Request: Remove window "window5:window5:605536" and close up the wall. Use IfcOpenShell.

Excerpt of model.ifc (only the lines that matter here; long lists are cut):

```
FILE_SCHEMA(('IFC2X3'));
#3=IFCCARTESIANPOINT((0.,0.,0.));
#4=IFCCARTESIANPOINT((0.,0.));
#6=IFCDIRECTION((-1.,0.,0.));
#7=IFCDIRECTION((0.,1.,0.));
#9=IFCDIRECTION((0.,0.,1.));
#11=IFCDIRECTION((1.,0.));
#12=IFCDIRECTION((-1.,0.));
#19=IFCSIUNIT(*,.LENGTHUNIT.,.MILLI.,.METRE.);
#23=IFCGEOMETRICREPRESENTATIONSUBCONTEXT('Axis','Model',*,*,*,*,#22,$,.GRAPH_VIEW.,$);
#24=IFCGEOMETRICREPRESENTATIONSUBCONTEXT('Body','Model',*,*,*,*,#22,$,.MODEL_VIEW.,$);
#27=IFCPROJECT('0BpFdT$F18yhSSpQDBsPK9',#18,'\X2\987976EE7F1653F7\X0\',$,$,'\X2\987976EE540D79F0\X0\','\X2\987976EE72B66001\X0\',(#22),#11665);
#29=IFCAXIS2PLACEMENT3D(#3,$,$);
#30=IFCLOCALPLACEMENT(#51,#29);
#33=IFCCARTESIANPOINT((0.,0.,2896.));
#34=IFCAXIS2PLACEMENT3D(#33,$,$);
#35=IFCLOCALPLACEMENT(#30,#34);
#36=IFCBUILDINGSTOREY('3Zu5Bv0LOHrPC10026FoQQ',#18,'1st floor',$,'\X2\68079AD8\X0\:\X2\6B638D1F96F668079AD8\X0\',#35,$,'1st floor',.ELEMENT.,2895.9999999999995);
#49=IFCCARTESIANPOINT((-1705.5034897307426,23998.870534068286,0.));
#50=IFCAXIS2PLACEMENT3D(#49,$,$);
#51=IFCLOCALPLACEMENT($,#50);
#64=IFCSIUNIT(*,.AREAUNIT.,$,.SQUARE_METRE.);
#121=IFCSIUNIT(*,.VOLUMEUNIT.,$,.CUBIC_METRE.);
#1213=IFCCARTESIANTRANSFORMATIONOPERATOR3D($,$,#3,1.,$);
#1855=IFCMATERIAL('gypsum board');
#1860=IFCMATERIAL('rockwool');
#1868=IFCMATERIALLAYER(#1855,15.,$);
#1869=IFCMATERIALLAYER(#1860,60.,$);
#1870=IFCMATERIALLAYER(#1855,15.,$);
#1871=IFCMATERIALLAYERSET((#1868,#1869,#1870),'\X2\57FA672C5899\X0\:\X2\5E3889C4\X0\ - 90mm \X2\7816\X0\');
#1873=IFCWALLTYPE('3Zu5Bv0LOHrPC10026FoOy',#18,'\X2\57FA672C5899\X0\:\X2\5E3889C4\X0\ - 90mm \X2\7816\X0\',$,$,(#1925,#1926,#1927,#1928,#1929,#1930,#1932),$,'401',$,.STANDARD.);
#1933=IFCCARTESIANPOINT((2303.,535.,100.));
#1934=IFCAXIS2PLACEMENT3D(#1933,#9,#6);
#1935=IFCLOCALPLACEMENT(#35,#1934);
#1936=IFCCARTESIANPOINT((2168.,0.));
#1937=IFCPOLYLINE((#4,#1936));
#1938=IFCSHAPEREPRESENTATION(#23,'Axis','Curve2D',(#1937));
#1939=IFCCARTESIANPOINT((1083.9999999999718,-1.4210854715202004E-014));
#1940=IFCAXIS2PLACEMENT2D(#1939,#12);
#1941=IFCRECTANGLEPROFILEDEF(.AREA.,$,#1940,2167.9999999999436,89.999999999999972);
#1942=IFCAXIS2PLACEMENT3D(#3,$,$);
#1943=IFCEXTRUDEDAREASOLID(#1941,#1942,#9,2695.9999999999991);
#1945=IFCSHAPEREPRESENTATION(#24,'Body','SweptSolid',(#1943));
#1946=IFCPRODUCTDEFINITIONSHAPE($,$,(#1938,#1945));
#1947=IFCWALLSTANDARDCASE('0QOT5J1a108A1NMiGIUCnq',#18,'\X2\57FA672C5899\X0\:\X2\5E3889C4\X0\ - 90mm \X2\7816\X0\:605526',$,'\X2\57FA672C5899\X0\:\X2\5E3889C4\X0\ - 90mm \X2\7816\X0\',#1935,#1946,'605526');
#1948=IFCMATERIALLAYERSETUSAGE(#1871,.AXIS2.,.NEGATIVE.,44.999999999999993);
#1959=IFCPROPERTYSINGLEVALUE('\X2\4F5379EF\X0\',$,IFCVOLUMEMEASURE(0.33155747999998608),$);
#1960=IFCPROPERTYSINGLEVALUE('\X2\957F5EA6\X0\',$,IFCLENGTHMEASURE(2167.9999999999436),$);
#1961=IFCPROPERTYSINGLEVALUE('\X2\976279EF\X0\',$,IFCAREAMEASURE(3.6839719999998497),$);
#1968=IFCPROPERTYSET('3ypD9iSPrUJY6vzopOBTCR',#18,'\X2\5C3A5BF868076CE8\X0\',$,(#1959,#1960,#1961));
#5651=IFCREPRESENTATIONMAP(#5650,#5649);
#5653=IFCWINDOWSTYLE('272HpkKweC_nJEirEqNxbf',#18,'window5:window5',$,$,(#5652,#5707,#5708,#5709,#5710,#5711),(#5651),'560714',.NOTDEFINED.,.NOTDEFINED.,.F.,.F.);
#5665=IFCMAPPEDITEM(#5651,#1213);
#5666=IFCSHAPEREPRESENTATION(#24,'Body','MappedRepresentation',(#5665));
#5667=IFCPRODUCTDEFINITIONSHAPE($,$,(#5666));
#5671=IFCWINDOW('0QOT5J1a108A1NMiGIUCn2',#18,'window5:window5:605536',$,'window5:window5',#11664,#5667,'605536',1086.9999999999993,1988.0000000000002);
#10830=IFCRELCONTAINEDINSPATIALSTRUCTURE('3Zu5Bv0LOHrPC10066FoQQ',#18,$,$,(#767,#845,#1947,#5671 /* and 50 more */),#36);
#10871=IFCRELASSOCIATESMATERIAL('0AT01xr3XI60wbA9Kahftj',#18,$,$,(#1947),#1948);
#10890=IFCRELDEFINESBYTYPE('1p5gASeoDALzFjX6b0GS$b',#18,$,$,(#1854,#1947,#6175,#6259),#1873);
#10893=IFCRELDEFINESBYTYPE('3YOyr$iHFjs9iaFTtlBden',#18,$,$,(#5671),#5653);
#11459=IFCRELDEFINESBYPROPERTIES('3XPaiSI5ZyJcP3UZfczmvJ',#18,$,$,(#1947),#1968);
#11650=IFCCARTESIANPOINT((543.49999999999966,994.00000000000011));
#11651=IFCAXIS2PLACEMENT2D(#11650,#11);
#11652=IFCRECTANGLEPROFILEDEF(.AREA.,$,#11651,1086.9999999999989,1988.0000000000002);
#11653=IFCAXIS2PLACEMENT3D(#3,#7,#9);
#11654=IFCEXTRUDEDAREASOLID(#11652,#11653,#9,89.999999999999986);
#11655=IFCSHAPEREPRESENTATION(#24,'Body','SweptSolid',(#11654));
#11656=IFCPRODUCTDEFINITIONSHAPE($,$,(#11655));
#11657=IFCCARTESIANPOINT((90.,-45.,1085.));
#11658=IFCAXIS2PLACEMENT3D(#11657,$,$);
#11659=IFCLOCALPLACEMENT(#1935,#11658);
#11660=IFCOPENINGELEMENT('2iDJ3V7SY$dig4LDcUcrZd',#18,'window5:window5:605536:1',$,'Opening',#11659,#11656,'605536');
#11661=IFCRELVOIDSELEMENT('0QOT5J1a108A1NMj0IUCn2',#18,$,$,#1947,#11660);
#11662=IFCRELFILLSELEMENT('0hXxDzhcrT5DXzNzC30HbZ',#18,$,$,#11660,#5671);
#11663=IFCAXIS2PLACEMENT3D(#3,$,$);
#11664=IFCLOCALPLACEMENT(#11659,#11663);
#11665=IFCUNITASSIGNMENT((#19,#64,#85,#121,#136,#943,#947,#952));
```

```python
import ifcopenshell
import ifcopenshell.api.feature
import ifcopenshell.api.pset
import ifcopenshell.api.root
import ifcopenshell.geom
import ifcopenshell.util.element
import ifcopenshell.util.shape
import ifcopenshell.util.unit

model = ifcopenshell.open("model.ifc")
area_scale = ifcopenshell.util.unit.calculate_unit_scale(model, "AREAUNIT")
volume_scale = ifcopenshell.util.unit.calculate_unit_scale(model, "VOLUMEUNIT")
settings = ifcopenshell.geom.settings()


def volume(element):
    """Net volume in cubic metres, openings subtracted."""
    shape = ifcopenshell.geom.create_shape(settings, element)
    return ifcopenshell.util.shape.get_volume(shape.geometry)


window = model.by_guid("0QOT5J1a108A1NMiGIUCn2")
opening = window.FillsVoids[0].RelatingOpeningElement
wall = opening.VoidsElements[0].RelatingBuildingElement
before = volume(wall)

ifcopenshell.api.root.remove_product(model, product=window)
ifcopenshell.api.feature.remove_feature(model, feature=opening)

after = volume(wall)
thickness = 0.09  # wall thickness in metres

# Update the wall's stored quantities.
pset = model.by_id(ifcopenshell.util.element.get_pset(wall, "尺寸标注", should_inherit=False)["id"])
ifcopenshell.api.pset.edit_pset(model, pset=pset, properties={
    "体积": model.create_entity("IfcVolumeMeasure", after / volume_scale),
    "面积": model.create_entity("IfcAreaMeasure", after / thickness / area_scale),
})

print(f"wall volume {before:.3f} -> {after:.3f} m3")

model.write("model-out.ifc")
```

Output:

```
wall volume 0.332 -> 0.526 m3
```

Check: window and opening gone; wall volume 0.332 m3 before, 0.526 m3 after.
